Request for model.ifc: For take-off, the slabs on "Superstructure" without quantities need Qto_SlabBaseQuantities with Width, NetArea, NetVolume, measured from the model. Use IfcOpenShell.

First a look at what the model holds.

```python
import ifcopenshell
import ifcopenshell.util.element
import ifcopenshell.util.unit

model = ifcopenshell.open("model.ifc")
print(model.schema)
for unit_type in ("LENGTHUNIT", "AREAUNIT", "VOLUMEUNIT"):
    print(unit_type, ifcopenshell.util.unit.calculate_unit_scale(model, unit_type))
storey = next(s for s in model.by_type("IfcBuildingStorey") if s.Name == "Superstructure")
slabs = [e for e in ifcopenshell.util.element.get_decomposition(storey) if e.is_a("IfcSlab")]
for e in sorted(slabs, key=lambda e: e.id()):
    print(e.id(), e.is_a(), e.Name, list(ifcopenshell.util.element.get_psets(e, qtos_only=True)), sep=" | ")
```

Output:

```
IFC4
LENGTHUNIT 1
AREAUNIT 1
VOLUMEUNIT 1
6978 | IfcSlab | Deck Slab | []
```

```python
import ifcopenshell
import ifcopenshell.api.pset
import ifcopenshell.geom
import ifcopenshell.util.element
import ifcopenshell.util.shape
import ifcopenshell.util.unit

model = ifcopenshell.open("model.ifc")
unit_scale = ifcopenshell.util.unit.calculate_unit_scale(model)
area_scale = ifcopenshell.util.unit.calculate_unit_scale(model, "AREAUNIT")
volume_scale = ifcopenshell.util.unit.calculate_unit_scale(model, "VOLUMEUNIT")
settings = ifcopenshell.geom.settings()

storey = next(s for s in model.by_type("IfcBuildingStorey") if s.Name == "Superstructure")
slabs = [e for e in ifcopenshell.util.element.get_decomposition(storey) if e.is_a("IfcSlab")]

for e in sorted(slabs, key=lambda e: e.id()):
    if ifcopenshell.util.element.get_psets(e, qtos_only=True, should_inherit=False):
        continue
    # Geometry comes back in metres, in the element's own axes.
    shape = ifcopenshell.geom.create_shape(settings, e)
    values = {
        "Width": ifcopenshell.util.shape.get_z(shape.geometry) / unit_scale,
        "NetArea": ifcopenshell.util.shape.get_footprint_area(shape.geometry) / area_scale,
        "NetVolume": ifcopenshell.util.shape.get_volume(shape.geometry) / volume_scale,
    }
    qto = ifcopenshell.api.pset.add_qto(model, product=e, name="Qto_SlabBaseQuantities")
    ifcopenshell.api.pset.edit_qto(model, qto=qto, properties=values)
    print(e.id(), {k: round(v, 3) for k, v in values.items()})

model.write("model-out.ifc")
```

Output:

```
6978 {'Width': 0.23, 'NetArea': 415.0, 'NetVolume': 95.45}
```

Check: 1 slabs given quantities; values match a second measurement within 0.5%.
